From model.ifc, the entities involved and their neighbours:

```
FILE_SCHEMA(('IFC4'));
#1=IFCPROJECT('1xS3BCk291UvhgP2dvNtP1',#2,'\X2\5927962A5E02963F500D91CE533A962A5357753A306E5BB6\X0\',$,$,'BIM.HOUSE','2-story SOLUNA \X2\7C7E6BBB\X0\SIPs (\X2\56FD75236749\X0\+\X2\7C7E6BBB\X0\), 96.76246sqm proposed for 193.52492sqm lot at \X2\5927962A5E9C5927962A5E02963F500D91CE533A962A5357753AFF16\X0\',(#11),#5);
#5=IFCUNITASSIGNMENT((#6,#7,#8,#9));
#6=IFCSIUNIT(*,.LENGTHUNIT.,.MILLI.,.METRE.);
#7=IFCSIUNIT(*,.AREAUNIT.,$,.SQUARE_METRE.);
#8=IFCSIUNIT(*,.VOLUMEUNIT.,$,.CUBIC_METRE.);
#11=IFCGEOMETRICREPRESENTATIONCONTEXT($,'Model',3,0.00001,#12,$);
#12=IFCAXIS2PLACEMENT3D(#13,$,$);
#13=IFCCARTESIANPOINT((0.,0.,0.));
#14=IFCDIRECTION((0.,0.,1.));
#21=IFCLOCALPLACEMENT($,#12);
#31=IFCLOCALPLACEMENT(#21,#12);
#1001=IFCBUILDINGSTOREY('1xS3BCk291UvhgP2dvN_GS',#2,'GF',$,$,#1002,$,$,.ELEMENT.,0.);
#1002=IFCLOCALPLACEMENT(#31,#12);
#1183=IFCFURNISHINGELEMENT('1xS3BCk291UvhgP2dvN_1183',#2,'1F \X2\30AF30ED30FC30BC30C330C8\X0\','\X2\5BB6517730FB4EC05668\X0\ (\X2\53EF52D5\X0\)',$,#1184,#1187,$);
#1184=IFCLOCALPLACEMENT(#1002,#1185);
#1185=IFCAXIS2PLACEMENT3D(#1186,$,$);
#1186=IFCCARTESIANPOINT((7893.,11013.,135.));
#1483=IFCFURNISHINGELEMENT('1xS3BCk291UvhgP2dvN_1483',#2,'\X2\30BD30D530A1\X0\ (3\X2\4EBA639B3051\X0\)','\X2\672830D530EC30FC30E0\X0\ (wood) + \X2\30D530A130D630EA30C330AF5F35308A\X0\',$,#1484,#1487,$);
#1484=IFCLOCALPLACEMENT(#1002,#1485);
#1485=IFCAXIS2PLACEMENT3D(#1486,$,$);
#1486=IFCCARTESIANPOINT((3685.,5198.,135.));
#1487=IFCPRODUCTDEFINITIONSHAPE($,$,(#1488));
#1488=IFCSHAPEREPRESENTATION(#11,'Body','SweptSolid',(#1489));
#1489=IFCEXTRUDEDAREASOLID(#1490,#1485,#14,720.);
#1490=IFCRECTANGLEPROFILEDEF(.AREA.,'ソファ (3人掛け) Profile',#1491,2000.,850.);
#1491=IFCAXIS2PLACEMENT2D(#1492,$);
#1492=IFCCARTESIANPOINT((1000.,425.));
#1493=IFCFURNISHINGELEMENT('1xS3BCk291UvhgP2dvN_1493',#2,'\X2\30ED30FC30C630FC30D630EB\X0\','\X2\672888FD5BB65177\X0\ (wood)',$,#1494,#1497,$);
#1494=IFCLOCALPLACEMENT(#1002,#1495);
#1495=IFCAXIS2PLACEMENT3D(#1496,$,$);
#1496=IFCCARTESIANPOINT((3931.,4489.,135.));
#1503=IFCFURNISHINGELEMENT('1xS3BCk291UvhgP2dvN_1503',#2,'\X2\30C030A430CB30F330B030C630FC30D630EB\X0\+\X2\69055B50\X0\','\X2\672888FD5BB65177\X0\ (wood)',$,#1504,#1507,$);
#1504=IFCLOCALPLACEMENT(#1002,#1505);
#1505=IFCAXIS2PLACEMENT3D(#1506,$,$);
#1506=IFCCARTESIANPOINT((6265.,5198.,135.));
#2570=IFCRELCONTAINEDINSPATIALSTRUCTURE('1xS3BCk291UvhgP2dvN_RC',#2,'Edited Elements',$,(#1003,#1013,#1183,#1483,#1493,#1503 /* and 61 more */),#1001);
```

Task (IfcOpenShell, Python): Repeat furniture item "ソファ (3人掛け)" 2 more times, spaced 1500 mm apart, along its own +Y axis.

```python
import ifcopenshell
import ifcopenshell.api.geometry
import ifcopenshell.api.root
import ifcopenshell.util.element
import ifcopenshell.util.placement

model = ifcopenshell.open("model.ifc")


def reuse_history(source, copy):
    """copy_class also copies each property set's owner history, people and application; keep the originals."""
    for rel in copy.IsDefinedBy:
        if rel.is_a("IfcRelDefinesByProperties") and (history := rel.RelatingPropertyDefinition.OwnerHistory):
            rel.RelatingPropertyDefinition.OwnerHistory = source.OwnerHistory
            ifcopenshell.util.element.remove_deep2(model, history)


source = model.by_id(1483)
base = ifcopenshell.util.placement.get_local_placement(source.ObjectPlacement)
step = base[:3, 1] * 1500.0

for i in range(1, 3):
    copy = ifcopenshell.api.root.copy_class(model, product=source)
    copy.Representation = ifcopenshell.util.element.copy_deep(
        model, source.Representation, exclude=["IfcGeometricRepresentationContext", "IfcRepresentationMap"]
    )
    reuse_history(source, copy)
    matrix = base.copy()
    matrix[:3, 3] += i * step
    print("added at", matrix[:3, 3].round(3) + 0.0)
    ifcopenshell.api.geometry.edit_object_placement(model, product=copy, matrix=matrix, is_si=False)

model.write("model_edited.ifc")
```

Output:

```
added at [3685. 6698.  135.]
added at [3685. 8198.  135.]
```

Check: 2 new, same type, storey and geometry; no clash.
